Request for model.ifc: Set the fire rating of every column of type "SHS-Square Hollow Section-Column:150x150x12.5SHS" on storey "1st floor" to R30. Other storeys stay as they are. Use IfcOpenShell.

First a look at what the model holds.

```python
import ifcopenshell
import ifcopenshell.util.element

model = ifcopenshell.open("model.ifc")
print(model.schema)
storey = next(s for s in model.by_type("IfcBuildingStorey") if s.Name == "1st floor")
columns = [e for e in ifcopenshell.util.element.get_decomposition(storey) if e.is_a("IfcColumn")]
seen = {}
for e in columns:
    element_type = ifcopenshell.util.element.get_type(e)
    key = (element_type.Name if element_type != e and element_type else None, ifcopenshell.util.element.get_pset(e, "Pset_ColumnCommon", "FireRating"))
    seen[key] = seen.get(key, 0) + 1
for (name, value), count in sorted(seen.items(), key=str):
    print(count, "x", name, "|", value)
```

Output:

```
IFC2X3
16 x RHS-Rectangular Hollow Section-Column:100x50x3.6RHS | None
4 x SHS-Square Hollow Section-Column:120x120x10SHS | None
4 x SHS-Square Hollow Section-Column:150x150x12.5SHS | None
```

```python
import ifcopenshell
import ifcopenshell.api.pset
import ifcopenshell.util.element

model = ifcopenshell.open("model.ifc")

storey = next(s for s in model.by_type("IfcBuildingStorey") if s.Name == "1st floor")
columns = [e for e in ifcopenshell.util.element.get_decomposition(storey) if e.is_a("IfcColumn")]

count = 0
for e in columns:
    element_type = ifcopenshell.util.element.get_type(e)
    if element_type in (None, e) or element_type.Name != "SHS-Square Hollow Section-Column:150x150x12.5SHS":
        continue
    # add_pset returns the element's existing set when there is one.
    pset = ifcopenshell.api.pset.add_pset(model, product=e, name="Pset_ColumnCommon")
    ifcopenshell.api.pset.edit_pset(model, pset=pset, properties={"FireRating": "R30"})
    count += 1

print(count, "columns updated")

model.write("model_v2.ifc")
```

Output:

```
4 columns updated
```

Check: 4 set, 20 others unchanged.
